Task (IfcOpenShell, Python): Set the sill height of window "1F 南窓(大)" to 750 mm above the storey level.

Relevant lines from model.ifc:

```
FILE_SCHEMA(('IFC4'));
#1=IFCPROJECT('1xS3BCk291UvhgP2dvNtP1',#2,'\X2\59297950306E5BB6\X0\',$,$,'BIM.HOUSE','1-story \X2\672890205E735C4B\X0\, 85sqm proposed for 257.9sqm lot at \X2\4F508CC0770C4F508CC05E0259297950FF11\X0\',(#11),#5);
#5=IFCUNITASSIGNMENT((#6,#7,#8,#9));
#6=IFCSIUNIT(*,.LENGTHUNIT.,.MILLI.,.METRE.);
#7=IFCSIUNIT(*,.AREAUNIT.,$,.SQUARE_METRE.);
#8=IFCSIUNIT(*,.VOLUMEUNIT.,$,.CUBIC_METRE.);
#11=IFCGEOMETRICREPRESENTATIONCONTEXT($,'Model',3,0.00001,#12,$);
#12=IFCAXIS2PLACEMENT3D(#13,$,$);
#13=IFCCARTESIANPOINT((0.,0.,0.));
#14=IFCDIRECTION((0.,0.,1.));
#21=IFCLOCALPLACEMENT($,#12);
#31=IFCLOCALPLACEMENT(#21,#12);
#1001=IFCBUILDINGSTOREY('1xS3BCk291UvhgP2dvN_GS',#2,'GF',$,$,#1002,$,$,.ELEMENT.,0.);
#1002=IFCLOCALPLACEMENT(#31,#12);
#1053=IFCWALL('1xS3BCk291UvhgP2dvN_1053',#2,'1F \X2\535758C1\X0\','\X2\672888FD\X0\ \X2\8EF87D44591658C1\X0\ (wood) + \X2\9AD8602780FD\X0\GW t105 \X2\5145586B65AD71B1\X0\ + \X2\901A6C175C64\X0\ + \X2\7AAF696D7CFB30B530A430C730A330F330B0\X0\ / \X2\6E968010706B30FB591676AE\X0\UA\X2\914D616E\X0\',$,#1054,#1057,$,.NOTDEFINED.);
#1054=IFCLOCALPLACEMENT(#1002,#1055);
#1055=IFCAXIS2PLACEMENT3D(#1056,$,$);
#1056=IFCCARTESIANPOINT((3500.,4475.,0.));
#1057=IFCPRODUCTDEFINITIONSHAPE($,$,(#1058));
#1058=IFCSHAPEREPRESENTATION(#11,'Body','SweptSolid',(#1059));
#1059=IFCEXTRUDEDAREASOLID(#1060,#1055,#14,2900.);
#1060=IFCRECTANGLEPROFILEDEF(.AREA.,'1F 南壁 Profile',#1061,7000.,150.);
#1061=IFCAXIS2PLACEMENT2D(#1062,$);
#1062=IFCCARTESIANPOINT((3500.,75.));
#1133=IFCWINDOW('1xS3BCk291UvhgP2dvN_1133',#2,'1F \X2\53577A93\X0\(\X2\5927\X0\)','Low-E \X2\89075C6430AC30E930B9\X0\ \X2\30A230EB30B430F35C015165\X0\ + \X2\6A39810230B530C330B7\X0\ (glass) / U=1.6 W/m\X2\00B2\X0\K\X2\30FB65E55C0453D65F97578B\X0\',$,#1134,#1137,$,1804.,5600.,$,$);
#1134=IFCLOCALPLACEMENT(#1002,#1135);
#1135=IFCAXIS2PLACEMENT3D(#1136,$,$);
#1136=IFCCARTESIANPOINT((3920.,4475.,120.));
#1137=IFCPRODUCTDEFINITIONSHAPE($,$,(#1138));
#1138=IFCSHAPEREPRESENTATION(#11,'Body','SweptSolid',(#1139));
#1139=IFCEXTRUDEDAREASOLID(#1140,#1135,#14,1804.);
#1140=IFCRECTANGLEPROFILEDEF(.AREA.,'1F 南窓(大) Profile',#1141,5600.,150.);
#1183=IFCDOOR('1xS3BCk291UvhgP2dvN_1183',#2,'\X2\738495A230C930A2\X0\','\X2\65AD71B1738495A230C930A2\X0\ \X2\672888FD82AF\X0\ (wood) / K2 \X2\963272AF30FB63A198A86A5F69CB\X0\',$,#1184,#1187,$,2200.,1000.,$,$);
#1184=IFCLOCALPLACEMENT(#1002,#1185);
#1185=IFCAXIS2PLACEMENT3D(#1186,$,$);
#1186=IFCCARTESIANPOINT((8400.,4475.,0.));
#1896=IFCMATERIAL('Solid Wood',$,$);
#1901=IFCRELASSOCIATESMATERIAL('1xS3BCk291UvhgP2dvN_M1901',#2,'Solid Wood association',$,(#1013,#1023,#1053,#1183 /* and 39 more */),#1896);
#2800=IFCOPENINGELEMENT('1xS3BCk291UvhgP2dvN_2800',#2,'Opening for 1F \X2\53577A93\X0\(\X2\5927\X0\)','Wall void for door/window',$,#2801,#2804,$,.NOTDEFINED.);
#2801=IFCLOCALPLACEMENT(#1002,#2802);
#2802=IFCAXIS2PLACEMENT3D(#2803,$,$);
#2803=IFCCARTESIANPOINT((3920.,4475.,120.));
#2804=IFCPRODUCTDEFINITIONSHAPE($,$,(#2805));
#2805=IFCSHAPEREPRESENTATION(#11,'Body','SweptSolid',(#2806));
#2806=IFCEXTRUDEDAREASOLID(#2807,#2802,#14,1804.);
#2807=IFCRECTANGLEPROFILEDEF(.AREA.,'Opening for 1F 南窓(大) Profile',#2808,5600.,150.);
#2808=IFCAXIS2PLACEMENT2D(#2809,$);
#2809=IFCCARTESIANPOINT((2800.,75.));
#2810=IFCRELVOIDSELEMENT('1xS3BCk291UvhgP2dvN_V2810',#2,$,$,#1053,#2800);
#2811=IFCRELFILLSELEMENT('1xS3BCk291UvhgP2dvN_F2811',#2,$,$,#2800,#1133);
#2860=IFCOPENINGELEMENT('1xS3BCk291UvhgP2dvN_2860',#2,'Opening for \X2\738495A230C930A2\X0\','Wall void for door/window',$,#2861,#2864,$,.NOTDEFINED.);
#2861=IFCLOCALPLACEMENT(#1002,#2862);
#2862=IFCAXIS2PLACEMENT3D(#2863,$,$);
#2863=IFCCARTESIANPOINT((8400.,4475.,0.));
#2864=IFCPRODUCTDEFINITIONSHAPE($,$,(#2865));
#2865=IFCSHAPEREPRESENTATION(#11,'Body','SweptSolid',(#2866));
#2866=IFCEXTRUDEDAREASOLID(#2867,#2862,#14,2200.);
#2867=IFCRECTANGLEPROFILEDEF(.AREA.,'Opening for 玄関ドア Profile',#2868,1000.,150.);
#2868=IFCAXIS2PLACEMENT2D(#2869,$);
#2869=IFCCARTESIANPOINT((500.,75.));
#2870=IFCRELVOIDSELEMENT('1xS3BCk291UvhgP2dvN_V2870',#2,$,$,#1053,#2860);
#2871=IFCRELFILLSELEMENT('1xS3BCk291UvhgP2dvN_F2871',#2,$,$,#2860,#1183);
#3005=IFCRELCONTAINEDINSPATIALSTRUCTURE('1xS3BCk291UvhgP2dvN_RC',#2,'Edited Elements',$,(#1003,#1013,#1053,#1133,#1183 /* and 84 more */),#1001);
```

```python
import numpy as np
import ifcopenshell
import ifcopenshell.api.geometry
import ifcopenshell.geom
import ifcopenshell.util.element
import ifcopenshell.util.placement
import ifcopenshell.util.shape
import ifcopenshell.util.unit

model = ifcopenshell.open("model.ifc")
unit_scale = ifcopenshell.util.unit.calculate_unit_scale(model)

window = model.by_id(1133)
opening = window.FillsVoids[0].RelatingOpeningElement
storey = ifcopenshell.util.element.get_container(window, ifc_class="IfcBuildingStorey")
level = ifcopenshell.util.placement.get_local_placement(storey.ObjectPlacement)[2, 3]

# The opening's origin need not be at the sill, so measure its lowest point.
shape = ifcopenshell.geom.create_shape(ifcopenshell.geom.settings(), opening)
bottom = ifcopenshell.util.shape.get_shape_bottom_elevation(shape, shape.geometry) / unit_scale
dz = level + 750.0 - bottom

shift = np.array([0.0, 0.0, dz])
# The window is not placed relative to its opening, so move both.
for product in (opening, window):
    matrix = ifcopenshell.util.placement.get_local_placement(product.ObjectPlacement)
    matrix[:3, 3] += shift
    ifcopenshell.api.geometry.edit_object_placement(model, product=product, matrix=matrix, is_si=False)

print(f"moved by {dz * unit_scale:+.3f} m")

model.write("model-out.ifc")
```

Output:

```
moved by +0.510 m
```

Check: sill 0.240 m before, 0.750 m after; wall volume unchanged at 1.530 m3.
